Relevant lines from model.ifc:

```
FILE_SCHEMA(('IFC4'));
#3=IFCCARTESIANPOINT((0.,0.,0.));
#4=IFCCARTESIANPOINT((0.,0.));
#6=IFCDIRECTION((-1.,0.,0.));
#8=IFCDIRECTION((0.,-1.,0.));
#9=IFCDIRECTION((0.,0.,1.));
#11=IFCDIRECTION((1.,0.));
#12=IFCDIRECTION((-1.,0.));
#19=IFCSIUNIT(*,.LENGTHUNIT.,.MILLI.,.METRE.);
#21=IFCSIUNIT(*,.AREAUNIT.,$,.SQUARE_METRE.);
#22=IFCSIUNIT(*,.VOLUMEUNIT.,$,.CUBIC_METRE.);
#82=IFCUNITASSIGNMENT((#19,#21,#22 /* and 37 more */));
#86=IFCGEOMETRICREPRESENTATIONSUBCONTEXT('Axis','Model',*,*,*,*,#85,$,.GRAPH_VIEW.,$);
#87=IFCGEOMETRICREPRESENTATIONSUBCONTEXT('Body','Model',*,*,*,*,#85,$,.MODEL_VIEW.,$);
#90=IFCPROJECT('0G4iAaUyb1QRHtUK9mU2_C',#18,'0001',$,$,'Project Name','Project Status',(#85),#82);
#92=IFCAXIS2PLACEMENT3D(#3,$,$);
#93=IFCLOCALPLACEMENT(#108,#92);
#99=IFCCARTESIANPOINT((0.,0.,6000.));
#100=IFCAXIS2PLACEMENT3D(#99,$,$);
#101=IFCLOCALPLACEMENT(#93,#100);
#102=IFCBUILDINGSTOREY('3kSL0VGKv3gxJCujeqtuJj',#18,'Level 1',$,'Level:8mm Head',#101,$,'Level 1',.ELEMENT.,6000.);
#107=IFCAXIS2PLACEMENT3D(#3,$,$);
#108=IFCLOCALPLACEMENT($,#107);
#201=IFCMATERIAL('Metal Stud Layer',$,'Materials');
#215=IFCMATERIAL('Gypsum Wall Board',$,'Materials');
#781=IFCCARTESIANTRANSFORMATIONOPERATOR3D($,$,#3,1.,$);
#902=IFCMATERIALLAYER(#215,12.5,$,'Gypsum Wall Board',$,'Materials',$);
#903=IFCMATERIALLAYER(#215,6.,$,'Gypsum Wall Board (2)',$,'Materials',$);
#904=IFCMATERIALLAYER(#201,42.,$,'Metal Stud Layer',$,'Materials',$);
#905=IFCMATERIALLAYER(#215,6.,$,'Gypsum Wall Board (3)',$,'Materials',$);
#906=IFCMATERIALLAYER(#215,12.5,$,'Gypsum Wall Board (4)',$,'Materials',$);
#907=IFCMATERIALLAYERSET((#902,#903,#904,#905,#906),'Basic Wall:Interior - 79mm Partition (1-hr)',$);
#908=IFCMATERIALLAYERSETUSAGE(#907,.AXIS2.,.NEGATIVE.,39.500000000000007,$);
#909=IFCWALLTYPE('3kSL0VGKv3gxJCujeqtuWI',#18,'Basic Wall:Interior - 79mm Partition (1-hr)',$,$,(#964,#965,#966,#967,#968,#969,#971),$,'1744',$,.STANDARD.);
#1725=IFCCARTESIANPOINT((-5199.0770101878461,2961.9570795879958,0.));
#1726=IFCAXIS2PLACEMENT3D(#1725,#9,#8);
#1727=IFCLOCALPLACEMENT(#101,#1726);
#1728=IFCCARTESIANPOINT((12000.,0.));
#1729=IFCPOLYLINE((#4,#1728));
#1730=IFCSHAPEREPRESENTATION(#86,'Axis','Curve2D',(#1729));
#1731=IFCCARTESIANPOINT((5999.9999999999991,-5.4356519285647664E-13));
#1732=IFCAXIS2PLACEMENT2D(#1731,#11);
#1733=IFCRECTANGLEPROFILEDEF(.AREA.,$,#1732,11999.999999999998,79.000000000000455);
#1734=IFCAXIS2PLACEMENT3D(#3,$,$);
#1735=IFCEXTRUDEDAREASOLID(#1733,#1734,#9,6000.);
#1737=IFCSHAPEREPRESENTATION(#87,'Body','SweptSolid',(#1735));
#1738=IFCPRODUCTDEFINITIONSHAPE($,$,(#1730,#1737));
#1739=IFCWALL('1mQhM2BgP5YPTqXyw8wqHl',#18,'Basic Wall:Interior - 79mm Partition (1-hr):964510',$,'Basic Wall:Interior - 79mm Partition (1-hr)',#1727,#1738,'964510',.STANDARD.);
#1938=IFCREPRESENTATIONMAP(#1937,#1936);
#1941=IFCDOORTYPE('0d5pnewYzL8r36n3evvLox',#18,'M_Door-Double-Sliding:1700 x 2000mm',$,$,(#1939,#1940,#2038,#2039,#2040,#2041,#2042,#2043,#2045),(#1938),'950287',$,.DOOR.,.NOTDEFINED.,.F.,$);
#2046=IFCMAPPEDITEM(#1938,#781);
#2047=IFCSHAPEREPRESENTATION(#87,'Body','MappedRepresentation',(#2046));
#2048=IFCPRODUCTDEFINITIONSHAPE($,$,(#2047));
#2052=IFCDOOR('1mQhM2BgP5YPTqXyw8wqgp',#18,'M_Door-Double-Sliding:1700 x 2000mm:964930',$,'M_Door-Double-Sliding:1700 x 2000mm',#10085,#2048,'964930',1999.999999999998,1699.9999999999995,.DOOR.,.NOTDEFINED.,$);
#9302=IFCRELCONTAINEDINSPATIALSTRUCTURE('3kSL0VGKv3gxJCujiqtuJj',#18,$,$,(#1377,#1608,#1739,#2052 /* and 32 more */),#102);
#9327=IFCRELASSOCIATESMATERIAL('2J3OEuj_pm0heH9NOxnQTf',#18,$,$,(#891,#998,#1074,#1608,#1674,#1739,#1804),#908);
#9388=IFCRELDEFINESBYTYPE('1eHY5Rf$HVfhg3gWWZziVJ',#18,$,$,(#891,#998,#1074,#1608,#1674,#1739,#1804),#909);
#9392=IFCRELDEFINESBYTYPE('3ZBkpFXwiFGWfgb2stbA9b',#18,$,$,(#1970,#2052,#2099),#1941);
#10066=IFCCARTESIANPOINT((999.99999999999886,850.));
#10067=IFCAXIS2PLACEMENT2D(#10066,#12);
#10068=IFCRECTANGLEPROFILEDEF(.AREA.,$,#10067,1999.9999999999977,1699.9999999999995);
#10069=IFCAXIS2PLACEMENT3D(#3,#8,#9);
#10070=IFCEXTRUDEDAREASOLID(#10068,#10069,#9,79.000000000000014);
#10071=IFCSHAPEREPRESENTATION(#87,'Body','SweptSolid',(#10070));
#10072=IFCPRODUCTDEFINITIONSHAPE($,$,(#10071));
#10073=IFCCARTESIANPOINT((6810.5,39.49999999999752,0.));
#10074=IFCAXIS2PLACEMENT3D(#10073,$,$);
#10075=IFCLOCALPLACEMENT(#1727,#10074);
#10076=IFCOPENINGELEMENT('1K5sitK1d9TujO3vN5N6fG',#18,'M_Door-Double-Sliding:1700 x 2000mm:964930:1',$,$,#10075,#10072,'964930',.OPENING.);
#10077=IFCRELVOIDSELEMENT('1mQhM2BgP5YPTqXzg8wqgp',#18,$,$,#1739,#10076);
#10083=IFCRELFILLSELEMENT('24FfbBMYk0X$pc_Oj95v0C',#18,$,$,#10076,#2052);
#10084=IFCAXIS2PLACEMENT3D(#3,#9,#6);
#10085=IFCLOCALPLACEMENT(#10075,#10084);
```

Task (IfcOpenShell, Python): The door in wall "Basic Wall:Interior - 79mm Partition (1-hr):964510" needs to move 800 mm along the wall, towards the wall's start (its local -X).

```python
import ifcopenshell
import ifcopenshell.api.geometry
import ifcopenshell.util.placement
import ifcopenshell.util.unit

model = ifcopenshell.open("model.ifc")
unit_scale = ifcopenshell.util.unit.calculate_unit_scale(model)

door = model.by_id(2052)
opening = door.FillsVoids[0].RelatingOpeningElement
wall = opening.VoidsElements[0].RelatingBuildingElement

wall_matrix = ifcopenshell.util.placement.get_local_placement(wall.ObjectPlacement)
shift = wall_matrix[:3, 0] * -0.8 / unit_scale
before = ifcopenshell.util.placement.get_local_placement(door.ObjectPlacement)[:3, 3].copy()

# The door is placed relative to its opening, so it follows when the opening moves.
matrix = ifcopenshell.util.placement.get_local_placement(opening.ObjectPlacement)
matrix[:3, 3] += shift
ifcopenshell.api.geometry.edit_object_placement(
    model, product=opening, matrix=matrix, is_si=False, should_transform_children=True
)

after = ifcopenshell.util.placement.get_local_placement(door.ObjectPlacement)[:3, 3]
print("door moved by", (after - before).round(3) + 0.0)

model.write("model_updated.ifc")
```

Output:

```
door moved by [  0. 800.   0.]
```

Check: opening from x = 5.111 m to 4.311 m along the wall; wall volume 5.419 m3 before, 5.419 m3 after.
